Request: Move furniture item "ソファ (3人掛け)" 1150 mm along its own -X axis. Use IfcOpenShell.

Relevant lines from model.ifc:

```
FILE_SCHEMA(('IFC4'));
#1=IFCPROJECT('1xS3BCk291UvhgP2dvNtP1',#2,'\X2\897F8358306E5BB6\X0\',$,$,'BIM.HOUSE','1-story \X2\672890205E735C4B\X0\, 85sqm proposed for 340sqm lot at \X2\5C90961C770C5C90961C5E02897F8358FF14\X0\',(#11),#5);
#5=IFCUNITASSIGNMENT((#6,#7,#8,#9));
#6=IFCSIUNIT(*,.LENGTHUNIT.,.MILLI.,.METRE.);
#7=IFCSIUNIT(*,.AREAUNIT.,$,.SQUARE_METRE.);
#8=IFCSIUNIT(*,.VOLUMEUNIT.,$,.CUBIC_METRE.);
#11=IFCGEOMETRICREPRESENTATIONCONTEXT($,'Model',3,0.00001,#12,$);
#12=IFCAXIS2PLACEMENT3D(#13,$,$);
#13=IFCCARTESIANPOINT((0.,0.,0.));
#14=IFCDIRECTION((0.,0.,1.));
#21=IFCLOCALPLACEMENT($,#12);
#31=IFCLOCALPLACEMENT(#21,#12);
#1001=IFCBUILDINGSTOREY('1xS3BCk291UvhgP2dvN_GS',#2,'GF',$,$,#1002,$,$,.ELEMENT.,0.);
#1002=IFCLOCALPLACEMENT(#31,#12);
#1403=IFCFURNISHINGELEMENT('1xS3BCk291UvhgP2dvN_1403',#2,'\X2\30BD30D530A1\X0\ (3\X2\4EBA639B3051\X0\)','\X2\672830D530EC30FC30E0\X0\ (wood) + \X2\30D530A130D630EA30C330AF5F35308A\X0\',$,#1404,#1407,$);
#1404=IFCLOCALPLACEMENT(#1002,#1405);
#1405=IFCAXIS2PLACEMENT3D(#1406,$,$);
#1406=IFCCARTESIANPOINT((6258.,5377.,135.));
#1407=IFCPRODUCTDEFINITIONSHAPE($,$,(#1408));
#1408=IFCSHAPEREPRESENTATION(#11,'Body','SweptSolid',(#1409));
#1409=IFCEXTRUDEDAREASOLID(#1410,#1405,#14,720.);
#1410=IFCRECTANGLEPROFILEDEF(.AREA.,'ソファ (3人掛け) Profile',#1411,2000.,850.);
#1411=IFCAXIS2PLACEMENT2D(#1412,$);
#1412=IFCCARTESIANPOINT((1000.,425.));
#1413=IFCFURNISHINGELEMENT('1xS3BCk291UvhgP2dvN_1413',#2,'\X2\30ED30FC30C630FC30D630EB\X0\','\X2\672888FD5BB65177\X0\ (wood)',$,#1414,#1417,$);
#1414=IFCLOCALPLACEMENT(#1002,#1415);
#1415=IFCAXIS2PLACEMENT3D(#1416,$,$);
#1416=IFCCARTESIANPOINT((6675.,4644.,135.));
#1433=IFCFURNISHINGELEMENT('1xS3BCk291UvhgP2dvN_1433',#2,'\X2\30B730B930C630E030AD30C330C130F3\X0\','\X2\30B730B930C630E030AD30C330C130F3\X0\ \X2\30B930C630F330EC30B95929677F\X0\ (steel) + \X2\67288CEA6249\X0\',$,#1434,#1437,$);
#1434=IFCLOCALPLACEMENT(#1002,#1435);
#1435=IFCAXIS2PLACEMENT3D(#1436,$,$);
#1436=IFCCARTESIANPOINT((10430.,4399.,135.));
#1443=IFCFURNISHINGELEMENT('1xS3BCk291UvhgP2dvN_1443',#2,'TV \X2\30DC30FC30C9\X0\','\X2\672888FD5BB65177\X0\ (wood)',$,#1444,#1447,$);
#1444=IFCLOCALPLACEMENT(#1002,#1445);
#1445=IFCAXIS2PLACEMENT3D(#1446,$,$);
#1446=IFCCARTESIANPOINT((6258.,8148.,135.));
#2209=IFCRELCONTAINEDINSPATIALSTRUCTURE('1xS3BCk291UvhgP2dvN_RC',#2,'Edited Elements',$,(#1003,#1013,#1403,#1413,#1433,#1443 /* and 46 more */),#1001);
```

```python
import ifcopenshell
import ifcopenshell.api.geometry
import ifcopenshell.util.placement

model = ifcopenshell.open("model.ifc")

item = model.by_guid("1xS3BCk291UvhgP2dvN_1403")
matrix = ifcopenshell.util.placement.get_local_placement(item.ObjectPlacement)
matrix[:3, 3] -= matrix[:3, 0] * 1150.0
ifcopenshell.api.geometry.edit_object_placement(model, product=item, matrix=matrix, is_si=False)

print(ifcopenshell.util.placement.get_local_placement(item.ObjectPlacement).round(3) + 0.0)

model.write("model_updated.ifc")
```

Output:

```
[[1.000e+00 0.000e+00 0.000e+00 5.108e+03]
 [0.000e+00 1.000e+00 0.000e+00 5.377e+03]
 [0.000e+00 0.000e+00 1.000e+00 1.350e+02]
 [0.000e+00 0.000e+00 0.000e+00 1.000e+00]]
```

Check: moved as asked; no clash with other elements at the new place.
